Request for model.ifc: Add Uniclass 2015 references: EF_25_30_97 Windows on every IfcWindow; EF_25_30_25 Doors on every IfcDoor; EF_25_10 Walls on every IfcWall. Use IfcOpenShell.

First a look at what the model holds.

```python
import ifcopenshell

model = ifcopenshell.open("model.ifc")
print(model.schema)
print("classifications:", [c.Name for c in model.by_type("IfcClassification")])
for ifc_class in ("IfcDoor", "IfcRoof", "IfcStair", "IfcWall", "IfcWindow"):
    print(ifc_class, len(model.by_type(ifc_class)))
```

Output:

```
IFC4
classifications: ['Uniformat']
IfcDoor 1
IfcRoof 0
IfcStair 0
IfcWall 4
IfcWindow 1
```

```python
import ifcopenshell
import ifcopenshell.api.classification

model = ifcopenshell.open("model.ifc")

system = ifcopenshell.api.classification.add_classification(model, classification="Uniclass 2015")

codes = {
    "IfcWindow": ("EF_25_30_97", "Windows"),
    "IfcDoor": ("EF_25_30_25", "Doors"),
    "IfcWall": ("EF_25_10", "Walls"),
}
for ifc_class, (code, name) in codes.items():
    products = model.by_type(ifc_class)
    ifcopenshell.api.classification.add_reference(
        model, products=products, classification=system, identification=code, name=name
    )
    print(code, len(products))

model.write("model-out.ifc")
```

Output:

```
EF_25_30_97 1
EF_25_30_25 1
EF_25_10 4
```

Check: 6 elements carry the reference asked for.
